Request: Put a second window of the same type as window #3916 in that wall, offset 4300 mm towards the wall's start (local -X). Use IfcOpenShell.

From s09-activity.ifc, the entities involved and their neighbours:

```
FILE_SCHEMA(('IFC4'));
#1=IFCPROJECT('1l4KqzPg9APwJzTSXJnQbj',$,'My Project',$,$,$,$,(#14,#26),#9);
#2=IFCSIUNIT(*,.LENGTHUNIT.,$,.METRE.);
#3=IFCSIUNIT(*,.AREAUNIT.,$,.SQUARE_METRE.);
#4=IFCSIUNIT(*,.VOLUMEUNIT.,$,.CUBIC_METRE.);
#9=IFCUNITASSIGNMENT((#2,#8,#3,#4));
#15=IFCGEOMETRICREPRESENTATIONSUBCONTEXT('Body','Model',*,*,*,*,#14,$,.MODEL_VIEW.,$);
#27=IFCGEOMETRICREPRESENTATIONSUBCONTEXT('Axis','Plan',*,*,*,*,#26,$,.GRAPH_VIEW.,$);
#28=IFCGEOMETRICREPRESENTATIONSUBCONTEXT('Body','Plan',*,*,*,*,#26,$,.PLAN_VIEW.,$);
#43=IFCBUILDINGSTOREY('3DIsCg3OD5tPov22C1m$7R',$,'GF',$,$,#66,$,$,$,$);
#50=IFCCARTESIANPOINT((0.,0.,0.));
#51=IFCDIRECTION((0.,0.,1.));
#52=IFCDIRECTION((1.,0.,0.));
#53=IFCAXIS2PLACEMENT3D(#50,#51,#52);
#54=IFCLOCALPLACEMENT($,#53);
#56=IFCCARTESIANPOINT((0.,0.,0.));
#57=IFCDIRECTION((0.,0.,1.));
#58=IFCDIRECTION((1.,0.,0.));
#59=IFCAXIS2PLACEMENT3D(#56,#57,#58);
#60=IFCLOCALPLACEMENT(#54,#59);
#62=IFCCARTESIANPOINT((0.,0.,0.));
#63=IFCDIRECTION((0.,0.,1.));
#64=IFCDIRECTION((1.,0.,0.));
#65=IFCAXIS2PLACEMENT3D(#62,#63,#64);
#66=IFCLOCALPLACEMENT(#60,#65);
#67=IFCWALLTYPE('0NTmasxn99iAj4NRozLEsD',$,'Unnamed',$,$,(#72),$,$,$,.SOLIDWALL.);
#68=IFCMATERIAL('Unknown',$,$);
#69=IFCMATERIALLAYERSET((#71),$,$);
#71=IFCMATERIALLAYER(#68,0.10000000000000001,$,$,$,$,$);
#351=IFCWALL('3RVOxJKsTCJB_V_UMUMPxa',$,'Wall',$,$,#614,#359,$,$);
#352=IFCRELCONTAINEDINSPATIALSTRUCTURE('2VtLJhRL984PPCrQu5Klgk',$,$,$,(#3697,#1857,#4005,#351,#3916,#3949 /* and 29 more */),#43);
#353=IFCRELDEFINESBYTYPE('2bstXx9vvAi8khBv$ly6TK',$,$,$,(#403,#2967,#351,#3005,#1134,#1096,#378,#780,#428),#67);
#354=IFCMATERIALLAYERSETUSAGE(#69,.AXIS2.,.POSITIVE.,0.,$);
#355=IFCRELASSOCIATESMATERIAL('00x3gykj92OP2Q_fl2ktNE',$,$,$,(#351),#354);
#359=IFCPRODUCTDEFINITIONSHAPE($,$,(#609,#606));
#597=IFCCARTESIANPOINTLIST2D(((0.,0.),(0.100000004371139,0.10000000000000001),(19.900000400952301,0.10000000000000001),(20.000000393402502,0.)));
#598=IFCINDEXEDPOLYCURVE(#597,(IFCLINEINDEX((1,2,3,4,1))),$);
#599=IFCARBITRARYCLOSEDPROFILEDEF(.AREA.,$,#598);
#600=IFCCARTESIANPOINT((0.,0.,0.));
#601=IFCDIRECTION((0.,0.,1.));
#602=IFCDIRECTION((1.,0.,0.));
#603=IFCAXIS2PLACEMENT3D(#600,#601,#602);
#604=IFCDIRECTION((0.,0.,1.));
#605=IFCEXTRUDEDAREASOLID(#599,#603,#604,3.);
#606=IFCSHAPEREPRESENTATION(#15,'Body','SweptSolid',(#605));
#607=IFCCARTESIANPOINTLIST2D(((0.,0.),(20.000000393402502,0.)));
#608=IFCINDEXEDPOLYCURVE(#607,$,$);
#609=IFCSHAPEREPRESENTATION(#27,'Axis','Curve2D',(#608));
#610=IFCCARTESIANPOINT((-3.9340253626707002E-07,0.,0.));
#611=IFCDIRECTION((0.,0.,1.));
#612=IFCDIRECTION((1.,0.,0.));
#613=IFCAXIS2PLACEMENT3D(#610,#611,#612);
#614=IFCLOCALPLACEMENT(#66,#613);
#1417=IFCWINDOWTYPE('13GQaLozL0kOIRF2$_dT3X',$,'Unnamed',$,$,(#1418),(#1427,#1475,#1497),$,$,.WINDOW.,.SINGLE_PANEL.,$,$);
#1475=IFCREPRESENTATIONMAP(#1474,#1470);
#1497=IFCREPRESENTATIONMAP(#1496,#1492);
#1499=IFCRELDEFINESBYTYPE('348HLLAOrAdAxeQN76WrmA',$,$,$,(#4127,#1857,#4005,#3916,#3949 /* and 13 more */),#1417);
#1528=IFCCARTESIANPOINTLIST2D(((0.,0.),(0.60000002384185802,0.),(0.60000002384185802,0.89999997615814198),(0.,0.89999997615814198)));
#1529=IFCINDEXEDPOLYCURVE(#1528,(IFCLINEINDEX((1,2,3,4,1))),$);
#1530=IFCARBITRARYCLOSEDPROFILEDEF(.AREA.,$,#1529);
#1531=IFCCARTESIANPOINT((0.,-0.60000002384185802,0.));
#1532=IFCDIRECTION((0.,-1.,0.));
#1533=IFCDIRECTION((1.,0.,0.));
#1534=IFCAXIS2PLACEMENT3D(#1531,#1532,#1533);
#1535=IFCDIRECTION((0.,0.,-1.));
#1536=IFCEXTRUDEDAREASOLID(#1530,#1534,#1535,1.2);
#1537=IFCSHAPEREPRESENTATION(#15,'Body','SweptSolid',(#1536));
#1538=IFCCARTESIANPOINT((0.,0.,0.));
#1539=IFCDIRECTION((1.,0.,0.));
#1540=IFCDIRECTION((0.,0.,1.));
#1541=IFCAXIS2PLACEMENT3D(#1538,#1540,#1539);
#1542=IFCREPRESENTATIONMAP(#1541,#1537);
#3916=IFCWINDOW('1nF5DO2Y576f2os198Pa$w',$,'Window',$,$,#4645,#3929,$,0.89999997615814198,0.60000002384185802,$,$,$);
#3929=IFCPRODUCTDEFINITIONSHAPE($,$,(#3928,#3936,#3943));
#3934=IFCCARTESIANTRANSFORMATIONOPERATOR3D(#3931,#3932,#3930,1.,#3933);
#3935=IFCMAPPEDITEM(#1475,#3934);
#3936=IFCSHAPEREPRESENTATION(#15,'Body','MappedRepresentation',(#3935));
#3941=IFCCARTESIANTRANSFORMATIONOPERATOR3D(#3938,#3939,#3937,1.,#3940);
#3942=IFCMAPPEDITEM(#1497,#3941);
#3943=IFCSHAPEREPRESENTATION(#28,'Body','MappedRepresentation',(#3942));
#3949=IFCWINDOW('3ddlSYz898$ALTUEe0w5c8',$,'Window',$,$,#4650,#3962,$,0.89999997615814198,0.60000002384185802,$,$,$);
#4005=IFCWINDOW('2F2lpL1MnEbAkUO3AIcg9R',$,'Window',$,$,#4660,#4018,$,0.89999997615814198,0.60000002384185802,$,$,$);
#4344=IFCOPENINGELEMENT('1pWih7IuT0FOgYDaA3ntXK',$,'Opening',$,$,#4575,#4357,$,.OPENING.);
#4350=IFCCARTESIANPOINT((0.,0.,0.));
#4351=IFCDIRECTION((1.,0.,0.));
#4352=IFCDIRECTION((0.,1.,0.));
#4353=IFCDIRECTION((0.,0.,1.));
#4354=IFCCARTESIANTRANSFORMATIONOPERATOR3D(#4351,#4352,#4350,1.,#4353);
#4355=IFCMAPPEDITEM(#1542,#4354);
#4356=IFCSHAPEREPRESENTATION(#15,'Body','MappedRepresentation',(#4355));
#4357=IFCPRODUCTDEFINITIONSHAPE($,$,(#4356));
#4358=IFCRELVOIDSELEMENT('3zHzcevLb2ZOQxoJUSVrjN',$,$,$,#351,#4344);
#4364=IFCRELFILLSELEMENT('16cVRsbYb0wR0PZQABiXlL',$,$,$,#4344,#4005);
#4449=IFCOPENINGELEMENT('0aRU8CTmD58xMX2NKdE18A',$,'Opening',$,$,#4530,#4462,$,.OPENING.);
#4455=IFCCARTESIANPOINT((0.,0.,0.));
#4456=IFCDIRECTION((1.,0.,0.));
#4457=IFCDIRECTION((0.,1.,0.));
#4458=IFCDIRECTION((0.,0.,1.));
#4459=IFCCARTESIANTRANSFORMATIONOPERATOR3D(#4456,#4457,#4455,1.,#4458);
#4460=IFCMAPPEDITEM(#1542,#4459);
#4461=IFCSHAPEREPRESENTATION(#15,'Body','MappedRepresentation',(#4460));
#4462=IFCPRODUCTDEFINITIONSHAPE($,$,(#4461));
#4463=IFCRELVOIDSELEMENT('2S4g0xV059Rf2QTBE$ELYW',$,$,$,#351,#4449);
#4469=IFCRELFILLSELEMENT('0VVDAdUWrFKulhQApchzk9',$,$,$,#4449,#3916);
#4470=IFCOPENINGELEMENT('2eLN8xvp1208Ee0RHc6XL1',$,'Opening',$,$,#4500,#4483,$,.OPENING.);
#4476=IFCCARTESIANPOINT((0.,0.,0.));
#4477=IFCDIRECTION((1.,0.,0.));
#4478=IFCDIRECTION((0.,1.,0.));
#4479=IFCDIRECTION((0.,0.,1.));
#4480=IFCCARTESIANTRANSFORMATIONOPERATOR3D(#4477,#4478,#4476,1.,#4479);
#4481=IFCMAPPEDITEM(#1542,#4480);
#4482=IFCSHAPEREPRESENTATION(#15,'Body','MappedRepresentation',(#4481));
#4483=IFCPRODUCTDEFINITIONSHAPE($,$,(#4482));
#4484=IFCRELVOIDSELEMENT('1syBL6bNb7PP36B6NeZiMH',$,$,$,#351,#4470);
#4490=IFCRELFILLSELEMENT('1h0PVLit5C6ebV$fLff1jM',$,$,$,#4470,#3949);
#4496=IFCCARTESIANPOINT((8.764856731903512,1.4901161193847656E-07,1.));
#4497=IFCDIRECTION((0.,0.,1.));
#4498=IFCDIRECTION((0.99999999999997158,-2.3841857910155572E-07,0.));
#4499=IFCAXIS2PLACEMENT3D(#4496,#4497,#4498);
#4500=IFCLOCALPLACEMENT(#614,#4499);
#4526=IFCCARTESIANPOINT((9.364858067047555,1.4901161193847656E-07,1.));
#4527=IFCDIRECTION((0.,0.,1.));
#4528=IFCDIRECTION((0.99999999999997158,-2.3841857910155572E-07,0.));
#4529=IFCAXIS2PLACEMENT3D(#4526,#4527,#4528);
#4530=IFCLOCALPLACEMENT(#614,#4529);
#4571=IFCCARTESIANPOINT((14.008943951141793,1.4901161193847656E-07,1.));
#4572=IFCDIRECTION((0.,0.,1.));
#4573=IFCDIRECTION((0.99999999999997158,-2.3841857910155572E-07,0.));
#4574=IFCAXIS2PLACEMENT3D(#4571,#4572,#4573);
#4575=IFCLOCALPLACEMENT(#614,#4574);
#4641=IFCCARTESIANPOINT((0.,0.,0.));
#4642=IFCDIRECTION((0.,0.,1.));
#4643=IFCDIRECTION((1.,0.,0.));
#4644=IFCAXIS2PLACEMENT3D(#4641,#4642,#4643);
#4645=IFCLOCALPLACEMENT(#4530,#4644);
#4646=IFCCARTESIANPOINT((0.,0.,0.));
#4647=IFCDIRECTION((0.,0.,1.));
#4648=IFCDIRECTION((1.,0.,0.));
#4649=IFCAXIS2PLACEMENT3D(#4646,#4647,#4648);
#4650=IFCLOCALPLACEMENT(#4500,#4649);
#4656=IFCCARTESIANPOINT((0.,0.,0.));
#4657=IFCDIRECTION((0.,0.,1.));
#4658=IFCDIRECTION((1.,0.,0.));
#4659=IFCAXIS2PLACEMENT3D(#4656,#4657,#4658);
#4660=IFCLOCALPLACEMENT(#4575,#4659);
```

```python
import ifcopenshell
import ifcopenshell.api.feature
import ifcopenshell.api.geometry
import ifcopenshell.api.root
import ifcopenshell.geom
import ifcopenshell.util.element
import ifcopenshell.util.placement
import ifcopenshell.util.shape
import ifcopenshell.util.unit

model = ifcopenshell.open("s09-activity.ifc")
unit_scale = ifcopenshell.util.unit.calculate_unit_scale(model)
settings = ifcopenshell.geom.settings()


def volume(element):
    """Net volume in cubic metres, openings subtracted."""
    shape = ifcopenshell.geom.create_shape(settings, element)
    return ifcopenshell.util.shape.get_volume(shape.geometry)


window = model.by_id(3916)
opening = window.FillsVoids[0].RelatingOpeningElement
wall = opening.VoidsElements[0].RelatingBuildingElement
before = volume(wall)
shift = ifcopenshell.util.placement.get_local_placement(wall.ObjectPlacement)[:3, 0] * -4.3 / unit_scale

# copy_class copies the void relationship, type, container and properties, but no geometry.
new_opening = ifcopenshell.api.root.copy_class(model, product=opening)
new_opening.Representation = ifcopenshell.util.element.copy_deep(
    model, opening.Representation, exclude=["IfcGeometricRepresentationContext", "IfcRepresentationMap"]
)
new_window = ifcopenshell.api.root.copy_class(model, product=window)
new_window.Representation = ifcopenshell.util.element.copy_deep(
    model, window.Representation, exclude=["IfcGeometricRepresentationContext", "IfcRepresentationMap"]
)
ifcopenshell.api.feature.add_filling(model, opening=new_opening, element=new_window)

for old, new in ((opening, new_opening), (window, new_window)):
    matrix = ifcopenshell.util.placement.get_local_placement(old.ObjectPlacement)
    matrix[:3, 3] += shift
    ifcopenshell.api.geometry.edit_object_placement(model, product=new, matrix=matrix, is_si=False)

after = volume(wall)

print(f"wall volume {before:.3f} -> {after:.3f} m3")

model.write("s09-activity_v2.ifc")
```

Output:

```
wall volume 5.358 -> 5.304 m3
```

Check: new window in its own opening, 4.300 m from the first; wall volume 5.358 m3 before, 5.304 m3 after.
